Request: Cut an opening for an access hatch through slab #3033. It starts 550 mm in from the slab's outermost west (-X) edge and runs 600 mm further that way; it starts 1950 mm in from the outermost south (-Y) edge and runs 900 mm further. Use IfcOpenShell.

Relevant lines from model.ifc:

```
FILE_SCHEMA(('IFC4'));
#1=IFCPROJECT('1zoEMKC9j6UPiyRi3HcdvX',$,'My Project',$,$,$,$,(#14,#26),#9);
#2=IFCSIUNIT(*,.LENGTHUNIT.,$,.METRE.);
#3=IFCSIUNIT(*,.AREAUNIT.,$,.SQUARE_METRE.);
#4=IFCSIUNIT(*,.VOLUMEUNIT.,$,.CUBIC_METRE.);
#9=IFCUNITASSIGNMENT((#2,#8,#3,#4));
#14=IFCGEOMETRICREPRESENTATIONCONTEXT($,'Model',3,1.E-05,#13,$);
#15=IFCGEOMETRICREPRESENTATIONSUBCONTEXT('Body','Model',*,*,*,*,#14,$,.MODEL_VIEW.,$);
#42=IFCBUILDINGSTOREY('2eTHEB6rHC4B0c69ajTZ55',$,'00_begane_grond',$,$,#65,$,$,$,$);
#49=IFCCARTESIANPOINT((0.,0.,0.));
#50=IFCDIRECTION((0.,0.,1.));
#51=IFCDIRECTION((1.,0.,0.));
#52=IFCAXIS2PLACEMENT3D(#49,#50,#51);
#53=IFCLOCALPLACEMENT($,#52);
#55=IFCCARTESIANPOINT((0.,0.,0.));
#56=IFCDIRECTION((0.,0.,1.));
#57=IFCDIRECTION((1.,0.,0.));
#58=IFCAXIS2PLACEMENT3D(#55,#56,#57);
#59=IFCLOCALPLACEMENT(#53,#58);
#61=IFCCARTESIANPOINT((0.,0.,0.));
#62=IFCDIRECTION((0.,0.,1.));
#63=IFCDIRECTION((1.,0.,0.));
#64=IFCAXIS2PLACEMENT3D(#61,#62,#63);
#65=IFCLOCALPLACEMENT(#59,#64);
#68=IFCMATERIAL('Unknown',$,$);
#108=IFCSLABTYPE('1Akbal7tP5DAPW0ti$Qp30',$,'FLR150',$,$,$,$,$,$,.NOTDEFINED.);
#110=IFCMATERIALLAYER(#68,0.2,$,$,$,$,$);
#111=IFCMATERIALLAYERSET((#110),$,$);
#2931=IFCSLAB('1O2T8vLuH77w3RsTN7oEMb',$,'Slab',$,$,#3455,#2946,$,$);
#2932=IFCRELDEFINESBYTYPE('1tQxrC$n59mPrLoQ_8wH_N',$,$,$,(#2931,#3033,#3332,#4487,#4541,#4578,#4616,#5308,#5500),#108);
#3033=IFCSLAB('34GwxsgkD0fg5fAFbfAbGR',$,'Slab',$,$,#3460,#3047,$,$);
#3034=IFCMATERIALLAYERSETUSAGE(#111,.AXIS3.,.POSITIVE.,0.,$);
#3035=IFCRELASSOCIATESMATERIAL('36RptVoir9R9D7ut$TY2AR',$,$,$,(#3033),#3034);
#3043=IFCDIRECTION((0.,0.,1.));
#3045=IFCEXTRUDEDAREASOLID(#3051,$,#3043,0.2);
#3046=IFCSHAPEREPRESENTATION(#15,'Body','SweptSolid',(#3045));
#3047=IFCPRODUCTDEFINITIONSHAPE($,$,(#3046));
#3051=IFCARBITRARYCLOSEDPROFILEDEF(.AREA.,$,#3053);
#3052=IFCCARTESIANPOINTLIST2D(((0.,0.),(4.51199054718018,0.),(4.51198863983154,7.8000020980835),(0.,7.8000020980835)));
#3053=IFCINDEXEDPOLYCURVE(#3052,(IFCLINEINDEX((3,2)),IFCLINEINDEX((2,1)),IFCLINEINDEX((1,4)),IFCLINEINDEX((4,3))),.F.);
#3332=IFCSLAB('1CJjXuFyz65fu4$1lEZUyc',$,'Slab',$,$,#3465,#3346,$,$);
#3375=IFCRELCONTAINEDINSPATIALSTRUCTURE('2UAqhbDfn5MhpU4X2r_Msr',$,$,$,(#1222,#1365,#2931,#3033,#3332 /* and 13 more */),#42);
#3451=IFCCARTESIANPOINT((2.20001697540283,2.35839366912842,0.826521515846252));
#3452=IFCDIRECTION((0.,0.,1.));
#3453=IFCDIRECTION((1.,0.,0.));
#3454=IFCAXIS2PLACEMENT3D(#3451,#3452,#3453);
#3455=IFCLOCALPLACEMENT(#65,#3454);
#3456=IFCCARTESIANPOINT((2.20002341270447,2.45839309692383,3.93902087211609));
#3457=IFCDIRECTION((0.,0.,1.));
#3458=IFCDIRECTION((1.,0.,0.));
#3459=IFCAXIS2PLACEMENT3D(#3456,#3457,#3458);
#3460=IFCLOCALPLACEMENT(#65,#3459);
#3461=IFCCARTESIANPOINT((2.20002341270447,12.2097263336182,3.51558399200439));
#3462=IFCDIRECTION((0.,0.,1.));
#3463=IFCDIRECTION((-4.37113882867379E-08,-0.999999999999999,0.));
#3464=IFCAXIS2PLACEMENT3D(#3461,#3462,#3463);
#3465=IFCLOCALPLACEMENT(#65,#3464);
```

```python
import numpy as np
import ifcopenshell
import ifcopenshell.api.feature
import ifcopenshell.api.geometry
import ifcopenshell.api.root
import ifcopenshell.geom
import ifcopenshell.util.placement
import ifcopenshell.util.representation
import ifcopenshell.util.shape
import ifcopenshell.util.unit

model = ifcopenshell.open("model.ifc")
unit_scale = ifcopenshell.util.unit.calculate_unit_scale(model)
settings = ifcopenshell.geom.settings()


def volume(element):
    """Net volume in cubic metres, openings subtracted."""
    shape = ifcopenshell.geom.create_shape(settings, element)
    return ifcopenshell.util.shape.get_volume(shape.geometry)


slab = model.by_guid("34GwxsgkD0fg5fAFbfAbGR")
before = volume(slab)

# Extent in the slab's own axes, in metres. The edges named are its -X and -Y sides.
slab_shape = ifcopenshell.geom.create_shape(settings, slab)
vertices = ifcopenshell.util.shape.get_vertices(slab_shape.geometry)
x_min, y_min, bottom = vertices.min(axis=0)
top = vertices[:, 2].max()

opening = ifcopenshell.api.root.create_entity(model, ifc_class="IfcOpeningElement", name="Access hatch opening", predefined_type="OPENING")
context = ifcopenshell.util.representation.get_context(model, "Model", "Body", "MODEL_VIEW")
width, depth = 0.6, 0.9
outline = [(0.0, 0.0), (width, 0.0), (width, depth), (0.0, depth), (0.0, 0.0)]
# Overshoot both faces by 50 mm so the cut is clean.
shape = ifcopenshell.api.geometry.add_slab_representation(
    model, context=context, depth=top - bottom + 0.1, polyline=outline
)
ifcopenshell.api.geometry.assign_representation(model, product=opening, representation=shape)

matrix = ifcopenshell.util.placement.get_local_placement(slab.ObjectPlacement)
matrix[:, 3] = matrix @ np.append(np.array([x_min + 0.55, y_min + 1.95, bottom - 0.05]) / unit_scale, 1.0)
ifcopenshell.api.geometry.edit_object_placement(model, product=opening, matrix=matrix, is_si=False)
ifcopenshell.api.feature.add_feature(model, feature=opening, element=slab)

after = volume(slab)

print(f"slab volume {before:.3f} -> {after:.3f} m3")

model.write("model_updated.ifc")
```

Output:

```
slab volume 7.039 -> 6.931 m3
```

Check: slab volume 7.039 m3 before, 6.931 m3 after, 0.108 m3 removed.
